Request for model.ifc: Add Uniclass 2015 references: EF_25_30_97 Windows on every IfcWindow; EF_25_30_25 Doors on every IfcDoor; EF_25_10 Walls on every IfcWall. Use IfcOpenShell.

First a look at what the model holds.

```python
import ifcopenshell

model = ifcopenshell.open("model.ifc")
print(model.schema)
print("classifications:", [c.Name for c in model.by_type("IfcClassification")])
for ifc_class in ("IfcDoor", "IfcRoof", "IfcStair", "IfcWall", "IfcWindow"):
    print(ifc_class, len(model.by_type(ifc_class)))
```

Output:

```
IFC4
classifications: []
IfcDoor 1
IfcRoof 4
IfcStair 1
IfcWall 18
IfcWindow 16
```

```python
import ifcopenshell
import ifcopenshell.api.classification

model = ifcopenshell.open("model.ifc")

system = ifcopenshell.api.classification.add_classification(model, classification="Uniclass 2015")

codes = {
    "IfcWindow": ("EF_25_30_97", "Windows"),
    "IfcDoor": ("EF_25_30_25", "Doors"),
    "IfcWall": ("EF_25_10", "Walls"),
}
for ifc_class, (code, name) in codes.items():
    products = model.by_type(ifc_class)
    ifcopenshell.api.classification.add_reference(
        model, products=products, classification=system, identification=code, name=name
    )
    print(code, len(products))

model.write("model_v2.ifc")
```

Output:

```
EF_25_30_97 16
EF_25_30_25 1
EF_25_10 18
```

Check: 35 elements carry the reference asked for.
